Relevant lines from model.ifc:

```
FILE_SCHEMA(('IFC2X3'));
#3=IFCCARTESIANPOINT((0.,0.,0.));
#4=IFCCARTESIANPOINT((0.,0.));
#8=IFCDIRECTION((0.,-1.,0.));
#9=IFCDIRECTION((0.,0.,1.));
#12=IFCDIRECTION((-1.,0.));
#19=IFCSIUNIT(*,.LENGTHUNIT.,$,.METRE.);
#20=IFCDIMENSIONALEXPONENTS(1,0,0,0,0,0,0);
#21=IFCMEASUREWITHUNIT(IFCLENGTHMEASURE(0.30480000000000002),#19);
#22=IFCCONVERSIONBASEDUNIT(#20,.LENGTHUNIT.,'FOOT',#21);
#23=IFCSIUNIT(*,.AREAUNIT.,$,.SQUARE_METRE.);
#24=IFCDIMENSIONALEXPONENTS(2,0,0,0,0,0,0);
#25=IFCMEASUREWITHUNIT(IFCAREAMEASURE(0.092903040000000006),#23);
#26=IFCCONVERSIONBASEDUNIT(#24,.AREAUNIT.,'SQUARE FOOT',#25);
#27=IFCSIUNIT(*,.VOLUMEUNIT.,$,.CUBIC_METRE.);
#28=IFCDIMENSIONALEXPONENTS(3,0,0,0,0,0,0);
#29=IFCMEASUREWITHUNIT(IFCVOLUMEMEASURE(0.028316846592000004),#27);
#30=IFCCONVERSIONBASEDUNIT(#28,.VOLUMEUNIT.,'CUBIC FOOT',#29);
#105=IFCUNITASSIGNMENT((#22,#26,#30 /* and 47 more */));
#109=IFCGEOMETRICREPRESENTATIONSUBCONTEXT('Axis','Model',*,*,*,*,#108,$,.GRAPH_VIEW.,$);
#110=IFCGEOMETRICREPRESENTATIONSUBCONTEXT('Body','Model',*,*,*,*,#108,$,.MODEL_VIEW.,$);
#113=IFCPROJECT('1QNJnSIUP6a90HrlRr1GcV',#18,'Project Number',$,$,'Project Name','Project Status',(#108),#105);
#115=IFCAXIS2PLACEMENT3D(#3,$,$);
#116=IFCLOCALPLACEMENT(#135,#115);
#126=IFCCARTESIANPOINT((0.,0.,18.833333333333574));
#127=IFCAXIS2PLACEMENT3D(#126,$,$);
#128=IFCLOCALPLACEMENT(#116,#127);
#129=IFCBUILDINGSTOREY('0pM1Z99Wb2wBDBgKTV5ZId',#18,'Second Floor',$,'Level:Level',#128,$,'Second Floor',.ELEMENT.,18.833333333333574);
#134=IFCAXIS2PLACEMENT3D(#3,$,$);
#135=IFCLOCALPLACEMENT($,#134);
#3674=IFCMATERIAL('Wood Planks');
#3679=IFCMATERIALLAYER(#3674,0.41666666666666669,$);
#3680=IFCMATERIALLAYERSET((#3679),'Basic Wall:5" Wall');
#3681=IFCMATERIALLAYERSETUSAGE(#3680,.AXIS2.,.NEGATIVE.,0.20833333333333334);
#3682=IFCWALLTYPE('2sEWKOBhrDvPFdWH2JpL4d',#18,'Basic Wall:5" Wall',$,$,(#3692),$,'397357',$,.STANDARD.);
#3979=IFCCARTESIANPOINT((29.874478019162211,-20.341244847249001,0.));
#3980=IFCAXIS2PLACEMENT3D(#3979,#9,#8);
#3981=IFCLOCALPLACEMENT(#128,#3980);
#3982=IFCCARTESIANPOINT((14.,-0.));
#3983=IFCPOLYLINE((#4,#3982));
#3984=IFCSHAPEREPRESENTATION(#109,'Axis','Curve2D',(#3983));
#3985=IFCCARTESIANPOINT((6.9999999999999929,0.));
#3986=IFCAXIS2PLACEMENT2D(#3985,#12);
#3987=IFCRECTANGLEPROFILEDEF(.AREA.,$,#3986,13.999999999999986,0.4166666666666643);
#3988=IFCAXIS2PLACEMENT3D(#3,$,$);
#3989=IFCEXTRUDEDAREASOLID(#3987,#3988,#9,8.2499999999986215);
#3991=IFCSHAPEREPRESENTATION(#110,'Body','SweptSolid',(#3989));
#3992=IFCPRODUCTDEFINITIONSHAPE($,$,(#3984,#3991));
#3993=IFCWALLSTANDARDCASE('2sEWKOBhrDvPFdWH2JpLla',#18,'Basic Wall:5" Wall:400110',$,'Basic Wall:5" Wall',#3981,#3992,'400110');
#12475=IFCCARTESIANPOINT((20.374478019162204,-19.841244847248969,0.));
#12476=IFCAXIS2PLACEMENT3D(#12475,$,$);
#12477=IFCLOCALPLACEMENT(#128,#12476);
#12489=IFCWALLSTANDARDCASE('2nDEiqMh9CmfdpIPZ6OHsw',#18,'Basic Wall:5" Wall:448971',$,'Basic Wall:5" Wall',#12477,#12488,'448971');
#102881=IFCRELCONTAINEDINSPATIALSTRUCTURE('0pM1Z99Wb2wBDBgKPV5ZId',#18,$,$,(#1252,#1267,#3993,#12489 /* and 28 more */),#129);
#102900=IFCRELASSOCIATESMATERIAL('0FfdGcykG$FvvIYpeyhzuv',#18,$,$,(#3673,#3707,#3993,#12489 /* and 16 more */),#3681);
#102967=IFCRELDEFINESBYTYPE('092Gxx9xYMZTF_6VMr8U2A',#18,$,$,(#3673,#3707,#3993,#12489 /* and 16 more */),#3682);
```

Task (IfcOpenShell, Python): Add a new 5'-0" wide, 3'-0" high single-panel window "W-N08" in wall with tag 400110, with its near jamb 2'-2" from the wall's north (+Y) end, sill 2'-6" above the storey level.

```python
import numpy as np
import ifcopenshell
import ifcopenshell.api.feature
import ifcopenshell.api.geometry
import ifcopenshell.api.root
import ifcopenshell.api.spatial
import ifcopenshell.api.type
import ifcopenshell.geom
import ifcopenshell.util.element
import ifcopenshell.util.placement
import ifcopenshell.util.representation
import ifcopenshell.util.shape
import ifcopenshell.util.unit

model = ifcopenshell.open("model.ifc")
unit_scale = ifcopenshell.util.unit.calculate_unit_scale(model)
settings = ifcopenshell.geom.settings()


def volume(element):
    """Net volume in cubic metres, openings subtracted."""
    shape = ifcopenshell.geom.create_shape(settings, element)
    return ifcopenshell.util.shape.get_volume(shape.geometry)


wall = model.by_guid("2sEWKOBhrDvPFdWH2JpLla")
storey = ifcopenshell.util.element.get_container(wall, ifc_class="IfcBuildingStorey")
context = ifcopenshell.util.representation.get_context(model, "Model", "Body", "MODEL_VIEW")
before = volume(wall)

width, height, from_end, sill = 1.524, 0.9144, 0.6604, 0.762  # metres

# The wall runs along its own X axis, and the end named is its -X end.
wall_shape = ifcopenshell.geom.create_shape(settings, wall)
x, y, z = ifcopenshell.util.shape.get_vertices(wall_shape.geometry).T
start = x.min() + from_end
face, thickness = float(y.min()), float(y.max() - y.min())
wall_matrix = ifcopenshell.util.placement.get_local_placement(wall.ObjectPlacement)
level = ifcopenshell.util.placement.get_local_placement(storey.ObjectPlacement)[2, 3]


def in_wall(x, y):
    """Placement at x, y metres in the wall's axes, at sill height."""
    matrix = wall_matrix.copy()
    matrix[:, 3] = wall_matrix @ np.array([x / unit_scale, y / unit_scale, 0.0, 1.0])
    matrix[2, 3] = level + sill / unit_scale
    return matrix


# Opening: a box that overshoots both wall faces by 50 mm.
opening = ifcopenshell.api.root.create_entity(model, ifc_class="IfcOpeningElement")
box = ifcopenshell.api.geometry.add_wall_representation(
    model, context=context, length=width, height=height, thickness=thickness + 0.1
)
ifcopenshell.api.geometry.assign_representation(model, product=opening, representation=box)
ifcopenshell.api.geometry.edit_object_placement(model, product=opening, matrix=in_wall(start, face - 0.05), is_si=False)
ifcopenshell.api.feature.add_feature(model, feature=opening, element=wall)

window = ifcopenshell.api.root.create_entity(model, ifc_class="IfcWindow", name="W-N08")
window.OverallWidth, window.OverallHeight = width / unit_scale, height / unit_scale
body = ifcopenshell.api.geometry.add_window_representation(
    model,
    context=context,
    overall_width=window.OverallWidth,
    overall_height=window.OverallHeight,
    partition_type="SINGLE_PANEL",
)
ifcopenshell.api.geometry.assign_representation(model, product=window, representation=body)
ifcopenshell.api.spatial.assign_container(model, products=[window], relating_structure=storey)
fills = ifcopenshell.api.feature.add_filling(model, opening=opening, element=window)
fills.OwnerHistory = window.OwnerHistory  # required in IFC2X3

# IFC2X3 keeps the operation on the window style.
style = ifcopenshell.api.root.create_entity(model, ifc_class="IfcWindowStyle", name="W-N08")
style.OperationType, style.ConstructionType = "SINGLE_PANEL", "NOTDEFINED"
style.ParameterTakesPrecedence = style.Sizeable = False
ifcopenshell.api.type.assign_type(model, related_objects=[window], relating_type=style)

# Centre the window in the wall's thickness.
ifcopenshell.api.geometry.edit_object_placement(model, product=window, matrix=in_wall(start, face), is_si=False)
window_shape = ifcopenshell.geom.create_shape(settings, window)
depth = ifcopenshell.util.shape.get_vertices(window_shape.geometry)[:, 1]
offset = face + thickness / 2 - (depth.min() + depth.max()) / 2
ifcopenshell.api.geometry.edit_object_placement(model, product=window, matrix=in_wall(start, offset), is_si=False)

after = volume(wall)

print(f"wall volume {before:.3f} -> {after:.3f} m3")

model.write("model_rev.ifc")
```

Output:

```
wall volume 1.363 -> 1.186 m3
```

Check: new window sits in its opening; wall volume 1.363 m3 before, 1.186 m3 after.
